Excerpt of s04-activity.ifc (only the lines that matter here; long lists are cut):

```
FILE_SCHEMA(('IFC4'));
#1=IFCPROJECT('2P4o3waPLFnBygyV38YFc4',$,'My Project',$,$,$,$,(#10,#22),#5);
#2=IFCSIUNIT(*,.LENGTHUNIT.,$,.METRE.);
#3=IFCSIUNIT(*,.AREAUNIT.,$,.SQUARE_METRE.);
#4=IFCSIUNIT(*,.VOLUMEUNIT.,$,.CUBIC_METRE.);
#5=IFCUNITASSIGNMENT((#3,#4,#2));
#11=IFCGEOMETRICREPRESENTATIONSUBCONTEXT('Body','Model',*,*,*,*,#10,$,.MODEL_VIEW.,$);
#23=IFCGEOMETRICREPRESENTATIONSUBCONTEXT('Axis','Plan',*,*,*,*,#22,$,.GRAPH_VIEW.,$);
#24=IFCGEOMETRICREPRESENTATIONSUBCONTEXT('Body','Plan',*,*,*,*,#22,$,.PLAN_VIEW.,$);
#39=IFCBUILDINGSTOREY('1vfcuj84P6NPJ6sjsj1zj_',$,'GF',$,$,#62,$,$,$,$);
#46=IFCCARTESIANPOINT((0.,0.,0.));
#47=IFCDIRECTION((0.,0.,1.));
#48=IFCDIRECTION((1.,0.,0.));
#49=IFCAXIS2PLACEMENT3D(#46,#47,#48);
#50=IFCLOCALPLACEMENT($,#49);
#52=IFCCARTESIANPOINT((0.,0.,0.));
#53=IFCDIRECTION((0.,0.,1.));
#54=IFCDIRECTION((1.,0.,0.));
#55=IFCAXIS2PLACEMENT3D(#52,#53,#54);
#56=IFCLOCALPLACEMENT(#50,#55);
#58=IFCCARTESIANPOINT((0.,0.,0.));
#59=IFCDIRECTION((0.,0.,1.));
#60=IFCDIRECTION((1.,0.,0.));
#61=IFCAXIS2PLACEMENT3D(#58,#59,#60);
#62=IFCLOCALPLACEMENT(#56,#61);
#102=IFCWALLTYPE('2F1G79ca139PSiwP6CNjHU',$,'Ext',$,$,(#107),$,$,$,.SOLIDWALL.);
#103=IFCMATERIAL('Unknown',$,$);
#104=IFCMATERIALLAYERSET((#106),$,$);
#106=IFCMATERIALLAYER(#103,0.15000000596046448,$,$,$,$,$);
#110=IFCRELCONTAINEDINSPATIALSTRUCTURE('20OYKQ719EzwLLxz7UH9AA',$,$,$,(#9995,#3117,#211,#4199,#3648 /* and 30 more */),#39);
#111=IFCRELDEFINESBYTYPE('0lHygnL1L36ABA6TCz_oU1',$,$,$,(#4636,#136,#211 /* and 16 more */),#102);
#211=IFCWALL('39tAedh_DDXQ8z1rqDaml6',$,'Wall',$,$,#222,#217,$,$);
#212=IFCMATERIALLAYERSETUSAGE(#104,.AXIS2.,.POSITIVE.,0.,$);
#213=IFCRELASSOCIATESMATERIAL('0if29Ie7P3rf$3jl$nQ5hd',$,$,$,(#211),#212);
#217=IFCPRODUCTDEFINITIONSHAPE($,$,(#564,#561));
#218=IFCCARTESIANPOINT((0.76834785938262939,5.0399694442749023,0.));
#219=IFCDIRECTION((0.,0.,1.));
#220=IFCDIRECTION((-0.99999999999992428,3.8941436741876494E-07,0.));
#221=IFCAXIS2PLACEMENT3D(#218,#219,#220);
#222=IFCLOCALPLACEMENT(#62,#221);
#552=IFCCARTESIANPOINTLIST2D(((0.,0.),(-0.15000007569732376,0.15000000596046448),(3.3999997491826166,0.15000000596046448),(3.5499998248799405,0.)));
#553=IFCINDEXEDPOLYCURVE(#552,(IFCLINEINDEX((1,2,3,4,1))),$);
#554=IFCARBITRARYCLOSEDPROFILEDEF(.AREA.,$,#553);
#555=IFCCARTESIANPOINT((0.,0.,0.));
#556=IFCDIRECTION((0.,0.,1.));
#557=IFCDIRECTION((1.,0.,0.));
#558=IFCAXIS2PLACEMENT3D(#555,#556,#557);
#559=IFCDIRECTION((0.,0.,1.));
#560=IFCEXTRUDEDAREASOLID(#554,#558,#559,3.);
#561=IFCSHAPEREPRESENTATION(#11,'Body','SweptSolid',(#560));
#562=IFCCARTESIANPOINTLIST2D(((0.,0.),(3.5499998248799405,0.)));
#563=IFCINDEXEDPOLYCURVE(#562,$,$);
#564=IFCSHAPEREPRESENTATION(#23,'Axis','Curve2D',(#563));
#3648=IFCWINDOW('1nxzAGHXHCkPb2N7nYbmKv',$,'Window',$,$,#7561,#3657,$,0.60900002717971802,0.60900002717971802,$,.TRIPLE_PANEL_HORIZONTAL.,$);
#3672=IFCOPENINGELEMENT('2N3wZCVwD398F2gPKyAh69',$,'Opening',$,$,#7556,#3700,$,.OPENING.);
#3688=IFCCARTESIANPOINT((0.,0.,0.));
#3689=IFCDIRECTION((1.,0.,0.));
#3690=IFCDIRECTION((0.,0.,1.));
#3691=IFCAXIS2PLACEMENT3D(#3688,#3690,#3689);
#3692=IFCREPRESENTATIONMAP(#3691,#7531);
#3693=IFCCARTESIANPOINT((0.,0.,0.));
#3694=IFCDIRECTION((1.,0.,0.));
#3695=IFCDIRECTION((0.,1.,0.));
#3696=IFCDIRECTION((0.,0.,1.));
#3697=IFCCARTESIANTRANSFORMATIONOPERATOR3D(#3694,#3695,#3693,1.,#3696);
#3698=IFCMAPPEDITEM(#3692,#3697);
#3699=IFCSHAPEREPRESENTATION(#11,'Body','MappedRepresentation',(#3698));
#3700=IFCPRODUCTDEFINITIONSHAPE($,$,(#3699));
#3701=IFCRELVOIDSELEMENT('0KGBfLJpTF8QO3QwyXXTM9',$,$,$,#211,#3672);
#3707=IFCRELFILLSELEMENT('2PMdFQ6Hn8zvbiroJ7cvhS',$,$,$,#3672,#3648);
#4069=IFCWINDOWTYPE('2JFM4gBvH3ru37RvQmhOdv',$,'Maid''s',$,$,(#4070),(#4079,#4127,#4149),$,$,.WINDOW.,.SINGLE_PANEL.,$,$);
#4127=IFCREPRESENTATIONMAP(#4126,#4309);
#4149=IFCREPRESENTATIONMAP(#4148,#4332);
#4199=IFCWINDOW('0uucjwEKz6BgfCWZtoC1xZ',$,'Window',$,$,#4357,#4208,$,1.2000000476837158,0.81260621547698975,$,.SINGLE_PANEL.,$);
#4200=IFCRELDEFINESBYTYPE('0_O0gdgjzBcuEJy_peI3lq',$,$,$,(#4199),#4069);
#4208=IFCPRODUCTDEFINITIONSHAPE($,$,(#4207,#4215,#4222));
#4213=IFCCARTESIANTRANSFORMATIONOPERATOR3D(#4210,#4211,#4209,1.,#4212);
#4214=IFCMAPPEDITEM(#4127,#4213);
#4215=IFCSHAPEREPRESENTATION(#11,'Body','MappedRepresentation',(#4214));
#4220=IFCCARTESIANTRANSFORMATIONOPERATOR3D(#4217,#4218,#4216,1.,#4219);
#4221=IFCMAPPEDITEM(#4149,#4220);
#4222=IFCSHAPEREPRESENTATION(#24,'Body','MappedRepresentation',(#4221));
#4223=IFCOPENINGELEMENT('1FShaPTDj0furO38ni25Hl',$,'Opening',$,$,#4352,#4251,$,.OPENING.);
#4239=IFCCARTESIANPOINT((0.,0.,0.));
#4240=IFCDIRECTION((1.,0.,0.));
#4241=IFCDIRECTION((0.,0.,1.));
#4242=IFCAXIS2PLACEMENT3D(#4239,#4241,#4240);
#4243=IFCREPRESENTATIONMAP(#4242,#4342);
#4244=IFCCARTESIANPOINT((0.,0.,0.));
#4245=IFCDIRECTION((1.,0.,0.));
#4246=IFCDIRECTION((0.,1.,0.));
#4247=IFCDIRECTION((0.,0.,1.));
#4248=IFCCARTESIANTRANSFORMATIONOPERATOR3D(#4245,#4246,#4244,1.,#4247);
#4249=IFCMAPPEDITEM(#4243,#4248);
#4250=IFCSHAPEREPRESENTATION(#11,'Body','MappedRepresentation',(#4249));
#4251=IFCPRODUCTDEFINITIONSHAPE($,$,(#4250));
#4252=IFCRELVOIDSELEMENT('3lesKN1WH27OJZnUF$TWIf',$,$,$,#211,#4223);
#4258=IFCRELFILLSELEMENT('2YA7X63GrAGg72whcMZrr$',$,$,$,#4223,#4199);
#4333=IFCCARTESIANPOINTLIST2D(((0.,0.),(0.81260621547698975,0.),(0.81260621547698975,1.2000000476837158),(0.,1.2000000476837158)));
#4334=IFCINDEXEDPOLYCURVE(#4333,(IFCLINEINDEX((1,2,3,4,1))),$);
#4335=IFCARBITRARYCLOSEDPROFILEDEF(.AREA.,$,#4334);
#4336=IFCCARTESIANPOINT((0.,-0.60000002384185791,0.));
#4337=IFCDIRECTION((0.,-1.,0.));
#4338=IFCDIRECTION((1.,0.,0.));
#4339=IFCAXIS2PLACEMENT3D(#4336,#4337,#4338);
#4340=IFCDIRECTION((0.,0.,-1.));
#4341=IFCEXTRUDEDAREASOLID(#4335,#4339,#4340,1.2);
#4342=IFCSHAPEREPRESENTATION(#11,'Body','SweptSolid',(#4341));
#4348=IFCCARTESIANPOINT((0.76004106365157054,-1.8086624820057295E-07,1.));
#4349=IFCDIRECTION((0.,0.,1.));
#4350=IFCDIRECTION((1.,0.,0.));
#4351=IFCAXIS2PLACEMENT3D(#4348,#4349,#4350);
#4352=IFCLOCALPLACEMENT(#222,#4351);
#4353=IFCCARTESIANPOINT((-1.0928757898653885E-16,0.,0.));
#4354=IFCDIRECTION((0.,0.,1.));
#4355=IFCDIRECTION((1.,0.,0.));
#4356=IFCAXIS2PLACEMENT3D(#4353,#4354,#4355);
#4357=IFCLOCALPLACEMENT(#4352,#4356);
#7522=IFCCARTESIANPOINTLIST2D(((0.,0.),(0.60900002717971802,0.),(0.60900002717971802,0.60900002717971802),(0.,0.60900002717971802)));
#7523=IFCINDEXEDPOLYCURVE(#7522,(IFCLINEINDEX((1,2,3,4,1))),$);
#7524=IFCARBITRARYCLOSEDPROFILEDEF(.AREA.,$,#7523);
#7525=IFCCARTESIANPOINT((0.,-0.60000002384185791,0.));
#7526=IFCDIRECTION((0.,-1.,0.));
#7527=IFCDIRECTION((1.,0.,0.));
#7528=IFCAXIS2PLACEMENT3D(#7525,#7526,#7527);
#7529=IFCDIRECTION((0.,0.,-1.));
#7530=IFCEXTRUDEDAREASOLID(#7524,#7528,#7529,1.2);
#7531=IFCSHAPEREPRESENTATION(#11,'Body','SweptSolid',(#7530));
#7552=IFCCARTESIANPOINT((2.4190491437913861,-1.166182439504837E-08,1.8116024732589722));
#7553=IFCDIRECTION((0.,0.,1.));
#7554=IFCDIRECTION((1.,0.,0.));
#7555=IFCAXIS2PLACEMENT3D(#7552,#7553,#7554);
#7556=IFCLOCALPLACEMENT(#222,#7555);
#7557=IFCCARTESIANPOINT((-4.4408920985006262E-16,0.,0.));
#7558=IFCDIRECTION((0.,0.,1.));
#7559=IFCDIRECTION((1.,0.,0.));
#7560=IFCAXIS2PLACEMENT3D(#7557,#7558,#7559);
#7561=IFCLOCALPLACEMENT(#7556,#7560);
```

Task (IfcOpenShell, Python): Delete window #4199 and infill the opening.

```python
import ifcopenshell
import ifcopenshell.api.feature
import ifcopenshell.api.root
import ifcopenshell.geom
import ifcopenshell.util.shape

model = ifcopenshell.open("s04-activity.ifc")
settings = ifcopenshell.geom.settings()


def volume(element):
    """Net volume in cubic metres, openings subtracted."""
    shape = ifcopenshell.geom.create_shape(settings, element)
    return ifcopenshell.util.shape.get_volume(shape.geometry)


window = model.by_guid("0uucjwEKz6BgfCWZtoC1xZ")
opening = window.FillsVoids[0].RelatingOpeningElement
wall = opening.VoidsElements[0].RelatingBuildingElement
before = volume(wall)

ifcopenshell.api.root.remove_product(model, product=window)
ifcopenshell.api.feature.remove_feature(model, feature=opening)

after = volume(wall)

print(f"wall volume {before:.3f} -> {after:.3f} m3")

model.write("s04-activity_updated.ifc")
```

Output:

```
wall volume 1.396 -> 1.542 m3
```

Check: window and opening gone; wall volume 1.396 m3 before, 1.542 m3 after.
